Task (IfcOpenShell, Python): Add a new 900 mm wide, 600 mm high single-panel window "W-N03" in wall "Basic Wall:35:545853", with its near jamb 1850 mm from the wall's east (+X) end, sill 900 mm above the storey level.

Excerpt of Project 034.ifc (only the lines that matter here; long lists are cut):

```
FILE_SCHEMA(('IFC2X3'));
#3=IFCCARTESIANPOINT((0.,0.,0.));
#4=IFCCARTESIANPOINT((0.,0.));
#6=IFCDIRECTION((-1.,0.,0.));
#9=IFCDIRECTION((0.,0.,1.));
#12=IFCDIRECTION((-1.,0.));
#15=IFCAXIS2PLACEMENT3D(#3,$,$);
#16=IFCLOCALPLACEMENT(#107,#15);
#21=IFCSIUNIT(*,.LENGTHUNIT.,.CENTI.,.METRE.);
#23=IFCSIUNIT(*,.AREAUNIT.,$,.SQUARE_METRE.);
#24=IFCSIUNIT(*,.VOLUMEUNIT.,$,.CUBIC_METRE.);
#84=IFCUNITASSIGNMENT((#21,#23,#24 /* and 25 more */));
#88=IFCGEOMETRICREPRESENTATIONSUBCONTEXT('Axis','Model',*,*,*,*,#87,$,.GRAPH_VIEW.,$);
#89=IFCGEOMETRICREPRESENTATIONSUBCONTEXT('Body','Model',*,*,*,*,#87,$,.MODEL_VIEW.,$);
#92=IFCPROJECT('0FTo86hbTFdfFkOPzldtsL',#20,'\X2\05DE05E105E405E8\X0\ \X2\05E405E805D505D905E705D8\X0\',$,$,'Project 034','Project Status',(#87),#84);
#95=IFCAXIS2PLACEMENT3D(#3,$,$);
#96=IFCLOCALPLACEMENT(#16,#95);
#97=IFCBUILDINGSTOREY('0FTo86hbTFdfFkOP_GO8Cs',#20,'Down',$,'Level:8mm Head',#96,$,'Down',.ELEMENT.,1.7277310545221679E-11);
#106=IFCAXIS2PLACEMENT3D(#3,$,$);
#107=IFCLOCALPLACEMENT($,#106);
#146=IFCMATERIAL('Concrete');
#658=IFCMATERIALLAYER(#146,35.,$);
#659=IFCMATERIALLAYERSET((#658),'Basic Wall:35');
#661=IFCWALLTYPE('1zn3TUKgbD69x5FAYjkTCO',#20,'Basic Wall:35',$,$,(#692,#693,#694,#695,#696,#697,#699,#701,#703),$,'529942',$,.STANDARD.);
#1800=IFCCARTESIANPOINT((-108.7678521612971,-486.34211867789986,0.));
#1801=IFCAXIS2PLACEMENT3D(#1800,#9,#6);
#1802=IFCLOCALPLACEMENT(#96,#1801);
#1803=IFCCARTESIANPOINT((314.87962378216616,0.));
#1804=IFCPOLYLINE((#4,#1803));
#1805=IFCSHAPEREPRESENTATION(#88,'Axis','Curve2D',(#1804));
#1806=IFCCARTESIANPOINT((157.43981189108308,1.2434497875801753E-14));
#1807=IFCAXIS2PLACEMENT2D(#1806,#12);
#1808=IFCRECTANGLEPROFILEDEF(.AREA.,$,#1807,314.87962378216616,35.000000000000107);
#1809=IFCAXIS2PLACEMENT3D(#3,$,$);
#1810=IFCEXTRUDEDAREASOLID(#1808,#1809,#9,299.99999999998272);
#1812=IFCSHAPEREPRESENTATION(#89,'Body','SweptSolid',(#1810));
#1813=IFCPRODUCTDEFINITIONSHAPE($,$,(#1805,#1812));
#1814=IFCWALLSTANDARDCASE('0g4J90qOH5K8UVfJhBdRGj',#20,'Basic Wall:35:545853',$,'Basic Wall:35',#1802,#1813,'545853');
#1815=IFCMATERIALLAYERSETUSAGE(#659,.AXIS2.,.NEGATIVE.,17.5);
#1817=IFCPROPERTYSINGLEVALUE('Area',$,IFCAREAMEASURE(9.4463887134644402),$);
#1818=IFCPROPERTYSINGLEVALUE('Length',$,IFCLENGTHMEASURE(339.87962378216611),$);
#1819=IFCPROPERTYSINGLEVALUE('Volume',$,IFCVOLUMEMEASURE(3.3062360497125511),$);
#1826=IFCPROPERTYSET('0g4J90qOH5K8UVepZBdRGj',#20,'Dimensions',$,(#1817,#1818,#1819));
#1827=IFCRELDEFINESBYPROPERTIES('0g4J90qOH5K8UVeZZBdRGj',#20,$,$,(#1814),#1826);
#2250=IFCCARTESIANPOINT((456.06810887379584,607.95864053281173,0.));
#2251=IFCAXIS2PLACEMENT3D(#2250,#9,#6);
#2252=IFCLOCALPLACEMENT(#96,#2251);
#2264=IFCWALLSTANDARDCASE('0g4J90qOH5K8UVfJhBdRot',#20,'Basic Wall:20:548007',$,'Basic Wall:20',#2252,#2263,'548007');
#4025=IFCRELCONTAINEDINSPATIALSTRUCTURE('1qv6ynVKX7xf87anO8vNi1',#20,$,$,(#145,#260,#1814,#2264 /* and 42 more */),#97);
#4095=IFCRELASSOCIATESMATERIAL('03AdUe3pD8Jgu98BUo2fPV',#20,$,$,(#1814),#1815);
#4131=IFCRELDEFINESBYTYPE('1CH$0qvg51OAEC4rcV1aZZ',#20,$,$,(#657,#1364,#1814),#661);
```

```python
import numpy as np
import ifcopenshell
import ifcopenshell.api.feature
import ifcopenshell.api.geometry
import ifcopenshell.api.pset
import ifcopenshell.api.root
import ifcopenshell.api.spatial
import ifcopenshell.api.type
import ifcopenshell.geom
import ifcopenshell.util.element
import ifcopenshell.util.placement
import ifcopenshell.util.representation
import ifcopenshell.util.shape
import ifcopenshell.util.unit

model = ifcopenshell.open("Project 034.ifc")
unit_scale = ifcopenshell.util.unit.calculate_unit_scale(model)
area_scale = ifcopenshell.util.unit.calculate_unit_scale(model, "AREAUNIT")
volume_scale = ifcopenshell.util.unit.calculate_unit_scale(model, "VOLUMEUNIT")
settings = ifcopenshell.geom.settings()


def volume(element):
    """Net volume in cubic metres, openings subtracted."""
    shape = ifcopenshell.geom.create_shape(settings, element)
    return ifcopenshell.util.shape.get_volume(shape.geometry)


wall = model.by_guid("0g4J90qOH5K8UVfJhBdRGj")
storey = ifcopenshell.util.element.get_container(wall, ifc_class="IfcBuildingStorey")
context = ifcopenshell.util.representation.get_context(model, "Model", "Body", "MODEL_VIEW")
before = volume(wall)

width, height, from_end, sill = 0.9, 0.6, 1.85, 0.9  # metres

# The wall runs along its own X axis, and the end named is its -X end.
wall_shape = ifcopenshell.geom.create_shape(settings, wall)
x, y, z = ifcopenshell.util.shape.get_vertices(wall_shape.geometry).T
start = x.min() + from_end
face, thickness = float(y.min()), float(y.max() - y.min())
wall_matrix = ifcopenshell.util.placement.get_local_placement(wall.ObjectPlacement)
level = ifcopenshell.util.placement.get_local_placement(storey.ObjectPlacement)[2, 3]


def in_wall(x, y):
    """Placement at x, y metres in the wall's axes, at sill height."""
    matrix = wall_matrix.copy()
    matrix[:, 3] = wall_matrix @ np.array([x / unit_scale, y / unit_scale, 0.0, 1.0])
    matrix[2, 3] = level + sill / unit_scale
    return matrix


# Opening: a box that overshoots both wall faces by 50 mm.
opening = ifcopenshell.api.root.create_entity(model, ifc_class="IfcOpeningElement")
box = ifcopenshell.api.geometry.add_wall_representation(
    model, context=context, length=width, height=height, thickness=thickness + 0.1
)
ifcopenshell.api.geometry.assign_representation(model, product=opening, representation=box)
ifcopenshell.api.geometry.edit_object_placement(model, product=opening, matrix=in_wall(start, face - 0.05), is_si=False)
ifcopenshell.api.feature.add_feature(model, feature=opening, element=wall)

window = ifcopenshell.api.root.create_entity(model, ifc_class="IfcWindow", name="W-N03")
window.OverallWidth, window.OverallHeight = width / unit_scale, height / unit_scale
body = ifcopenshell.api.geometry.add_window_representation(
    model,
    context=context,
    overall_width=window.OverallWidth,
    overall_height=window.OverallHeight,
    partition_type="SINGLE_PANEL",
)
ifcopenshell.api.geometry.assign_representation(model, product=window, representation=body)
ifcopenshell.api.spatial.assign_container(model, products=[window], relating_structure=storey)
fills = ifcopenshell.api.feature.add_filling(model, opening=opening, element=window)
fills.OwnerHistory = window.OwnerHistory  # required in IFC2X3

# IFC2X3 keeps the operation on the window style.
style = ifcopenshell.api.root.create_entity(model, ifc_class="IfcWindowStyle", name="W-N03")
style.OperationType, style.ConstructionType = "SINGLE_PANEL", "NOTDEFINED"
style.ParameterTakesPrecedence = style.Sizeable = False
ifcopenshell.api.type.assign_type(model, related_objects=[window], relating_type=style)

# Centre the window in the wall's thickness.
ifcopenshell.api.geometry.edit_object_placement(model, product=window, matrix=in_wall(start, face), is_si=False)
window_shape = ifcopenshell.geom.create_shape(settings, window)
depth = ifcopenshell.util.shape.get_vertices(window_shape.geometry)[:, 1]
offset = face + thickness / 2 - (depth.min() + depth.max()) / 2
ifcopenshell.api.geometry.edit_object_placement(model, product=window, matrix=in_wall(start, offset), is_si=False)

after = volume(wall)

# Update the wall's stored quantities.
pset = model.by_id(ifcopenshell.util.element.get_pset(wall, "Dimensions", should_inherit=False)["id"])
ifcopenshell.api.pset.edit_pset(model, pset=pset, properties={
    "Area": model.create_entity("IfcAreaMeasure", after / thickness / area_scale),
    "Volume": model.create_entity("IfcVolumeMeasure", after / volume_scale),
})

print(f"wall volume {before:.3f} -> {after:.3f} m3")

model.write("Project 034-out.ifc")
```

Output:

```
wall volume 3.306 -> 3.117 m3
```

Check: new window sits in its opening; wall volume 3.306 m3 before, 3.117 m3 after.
